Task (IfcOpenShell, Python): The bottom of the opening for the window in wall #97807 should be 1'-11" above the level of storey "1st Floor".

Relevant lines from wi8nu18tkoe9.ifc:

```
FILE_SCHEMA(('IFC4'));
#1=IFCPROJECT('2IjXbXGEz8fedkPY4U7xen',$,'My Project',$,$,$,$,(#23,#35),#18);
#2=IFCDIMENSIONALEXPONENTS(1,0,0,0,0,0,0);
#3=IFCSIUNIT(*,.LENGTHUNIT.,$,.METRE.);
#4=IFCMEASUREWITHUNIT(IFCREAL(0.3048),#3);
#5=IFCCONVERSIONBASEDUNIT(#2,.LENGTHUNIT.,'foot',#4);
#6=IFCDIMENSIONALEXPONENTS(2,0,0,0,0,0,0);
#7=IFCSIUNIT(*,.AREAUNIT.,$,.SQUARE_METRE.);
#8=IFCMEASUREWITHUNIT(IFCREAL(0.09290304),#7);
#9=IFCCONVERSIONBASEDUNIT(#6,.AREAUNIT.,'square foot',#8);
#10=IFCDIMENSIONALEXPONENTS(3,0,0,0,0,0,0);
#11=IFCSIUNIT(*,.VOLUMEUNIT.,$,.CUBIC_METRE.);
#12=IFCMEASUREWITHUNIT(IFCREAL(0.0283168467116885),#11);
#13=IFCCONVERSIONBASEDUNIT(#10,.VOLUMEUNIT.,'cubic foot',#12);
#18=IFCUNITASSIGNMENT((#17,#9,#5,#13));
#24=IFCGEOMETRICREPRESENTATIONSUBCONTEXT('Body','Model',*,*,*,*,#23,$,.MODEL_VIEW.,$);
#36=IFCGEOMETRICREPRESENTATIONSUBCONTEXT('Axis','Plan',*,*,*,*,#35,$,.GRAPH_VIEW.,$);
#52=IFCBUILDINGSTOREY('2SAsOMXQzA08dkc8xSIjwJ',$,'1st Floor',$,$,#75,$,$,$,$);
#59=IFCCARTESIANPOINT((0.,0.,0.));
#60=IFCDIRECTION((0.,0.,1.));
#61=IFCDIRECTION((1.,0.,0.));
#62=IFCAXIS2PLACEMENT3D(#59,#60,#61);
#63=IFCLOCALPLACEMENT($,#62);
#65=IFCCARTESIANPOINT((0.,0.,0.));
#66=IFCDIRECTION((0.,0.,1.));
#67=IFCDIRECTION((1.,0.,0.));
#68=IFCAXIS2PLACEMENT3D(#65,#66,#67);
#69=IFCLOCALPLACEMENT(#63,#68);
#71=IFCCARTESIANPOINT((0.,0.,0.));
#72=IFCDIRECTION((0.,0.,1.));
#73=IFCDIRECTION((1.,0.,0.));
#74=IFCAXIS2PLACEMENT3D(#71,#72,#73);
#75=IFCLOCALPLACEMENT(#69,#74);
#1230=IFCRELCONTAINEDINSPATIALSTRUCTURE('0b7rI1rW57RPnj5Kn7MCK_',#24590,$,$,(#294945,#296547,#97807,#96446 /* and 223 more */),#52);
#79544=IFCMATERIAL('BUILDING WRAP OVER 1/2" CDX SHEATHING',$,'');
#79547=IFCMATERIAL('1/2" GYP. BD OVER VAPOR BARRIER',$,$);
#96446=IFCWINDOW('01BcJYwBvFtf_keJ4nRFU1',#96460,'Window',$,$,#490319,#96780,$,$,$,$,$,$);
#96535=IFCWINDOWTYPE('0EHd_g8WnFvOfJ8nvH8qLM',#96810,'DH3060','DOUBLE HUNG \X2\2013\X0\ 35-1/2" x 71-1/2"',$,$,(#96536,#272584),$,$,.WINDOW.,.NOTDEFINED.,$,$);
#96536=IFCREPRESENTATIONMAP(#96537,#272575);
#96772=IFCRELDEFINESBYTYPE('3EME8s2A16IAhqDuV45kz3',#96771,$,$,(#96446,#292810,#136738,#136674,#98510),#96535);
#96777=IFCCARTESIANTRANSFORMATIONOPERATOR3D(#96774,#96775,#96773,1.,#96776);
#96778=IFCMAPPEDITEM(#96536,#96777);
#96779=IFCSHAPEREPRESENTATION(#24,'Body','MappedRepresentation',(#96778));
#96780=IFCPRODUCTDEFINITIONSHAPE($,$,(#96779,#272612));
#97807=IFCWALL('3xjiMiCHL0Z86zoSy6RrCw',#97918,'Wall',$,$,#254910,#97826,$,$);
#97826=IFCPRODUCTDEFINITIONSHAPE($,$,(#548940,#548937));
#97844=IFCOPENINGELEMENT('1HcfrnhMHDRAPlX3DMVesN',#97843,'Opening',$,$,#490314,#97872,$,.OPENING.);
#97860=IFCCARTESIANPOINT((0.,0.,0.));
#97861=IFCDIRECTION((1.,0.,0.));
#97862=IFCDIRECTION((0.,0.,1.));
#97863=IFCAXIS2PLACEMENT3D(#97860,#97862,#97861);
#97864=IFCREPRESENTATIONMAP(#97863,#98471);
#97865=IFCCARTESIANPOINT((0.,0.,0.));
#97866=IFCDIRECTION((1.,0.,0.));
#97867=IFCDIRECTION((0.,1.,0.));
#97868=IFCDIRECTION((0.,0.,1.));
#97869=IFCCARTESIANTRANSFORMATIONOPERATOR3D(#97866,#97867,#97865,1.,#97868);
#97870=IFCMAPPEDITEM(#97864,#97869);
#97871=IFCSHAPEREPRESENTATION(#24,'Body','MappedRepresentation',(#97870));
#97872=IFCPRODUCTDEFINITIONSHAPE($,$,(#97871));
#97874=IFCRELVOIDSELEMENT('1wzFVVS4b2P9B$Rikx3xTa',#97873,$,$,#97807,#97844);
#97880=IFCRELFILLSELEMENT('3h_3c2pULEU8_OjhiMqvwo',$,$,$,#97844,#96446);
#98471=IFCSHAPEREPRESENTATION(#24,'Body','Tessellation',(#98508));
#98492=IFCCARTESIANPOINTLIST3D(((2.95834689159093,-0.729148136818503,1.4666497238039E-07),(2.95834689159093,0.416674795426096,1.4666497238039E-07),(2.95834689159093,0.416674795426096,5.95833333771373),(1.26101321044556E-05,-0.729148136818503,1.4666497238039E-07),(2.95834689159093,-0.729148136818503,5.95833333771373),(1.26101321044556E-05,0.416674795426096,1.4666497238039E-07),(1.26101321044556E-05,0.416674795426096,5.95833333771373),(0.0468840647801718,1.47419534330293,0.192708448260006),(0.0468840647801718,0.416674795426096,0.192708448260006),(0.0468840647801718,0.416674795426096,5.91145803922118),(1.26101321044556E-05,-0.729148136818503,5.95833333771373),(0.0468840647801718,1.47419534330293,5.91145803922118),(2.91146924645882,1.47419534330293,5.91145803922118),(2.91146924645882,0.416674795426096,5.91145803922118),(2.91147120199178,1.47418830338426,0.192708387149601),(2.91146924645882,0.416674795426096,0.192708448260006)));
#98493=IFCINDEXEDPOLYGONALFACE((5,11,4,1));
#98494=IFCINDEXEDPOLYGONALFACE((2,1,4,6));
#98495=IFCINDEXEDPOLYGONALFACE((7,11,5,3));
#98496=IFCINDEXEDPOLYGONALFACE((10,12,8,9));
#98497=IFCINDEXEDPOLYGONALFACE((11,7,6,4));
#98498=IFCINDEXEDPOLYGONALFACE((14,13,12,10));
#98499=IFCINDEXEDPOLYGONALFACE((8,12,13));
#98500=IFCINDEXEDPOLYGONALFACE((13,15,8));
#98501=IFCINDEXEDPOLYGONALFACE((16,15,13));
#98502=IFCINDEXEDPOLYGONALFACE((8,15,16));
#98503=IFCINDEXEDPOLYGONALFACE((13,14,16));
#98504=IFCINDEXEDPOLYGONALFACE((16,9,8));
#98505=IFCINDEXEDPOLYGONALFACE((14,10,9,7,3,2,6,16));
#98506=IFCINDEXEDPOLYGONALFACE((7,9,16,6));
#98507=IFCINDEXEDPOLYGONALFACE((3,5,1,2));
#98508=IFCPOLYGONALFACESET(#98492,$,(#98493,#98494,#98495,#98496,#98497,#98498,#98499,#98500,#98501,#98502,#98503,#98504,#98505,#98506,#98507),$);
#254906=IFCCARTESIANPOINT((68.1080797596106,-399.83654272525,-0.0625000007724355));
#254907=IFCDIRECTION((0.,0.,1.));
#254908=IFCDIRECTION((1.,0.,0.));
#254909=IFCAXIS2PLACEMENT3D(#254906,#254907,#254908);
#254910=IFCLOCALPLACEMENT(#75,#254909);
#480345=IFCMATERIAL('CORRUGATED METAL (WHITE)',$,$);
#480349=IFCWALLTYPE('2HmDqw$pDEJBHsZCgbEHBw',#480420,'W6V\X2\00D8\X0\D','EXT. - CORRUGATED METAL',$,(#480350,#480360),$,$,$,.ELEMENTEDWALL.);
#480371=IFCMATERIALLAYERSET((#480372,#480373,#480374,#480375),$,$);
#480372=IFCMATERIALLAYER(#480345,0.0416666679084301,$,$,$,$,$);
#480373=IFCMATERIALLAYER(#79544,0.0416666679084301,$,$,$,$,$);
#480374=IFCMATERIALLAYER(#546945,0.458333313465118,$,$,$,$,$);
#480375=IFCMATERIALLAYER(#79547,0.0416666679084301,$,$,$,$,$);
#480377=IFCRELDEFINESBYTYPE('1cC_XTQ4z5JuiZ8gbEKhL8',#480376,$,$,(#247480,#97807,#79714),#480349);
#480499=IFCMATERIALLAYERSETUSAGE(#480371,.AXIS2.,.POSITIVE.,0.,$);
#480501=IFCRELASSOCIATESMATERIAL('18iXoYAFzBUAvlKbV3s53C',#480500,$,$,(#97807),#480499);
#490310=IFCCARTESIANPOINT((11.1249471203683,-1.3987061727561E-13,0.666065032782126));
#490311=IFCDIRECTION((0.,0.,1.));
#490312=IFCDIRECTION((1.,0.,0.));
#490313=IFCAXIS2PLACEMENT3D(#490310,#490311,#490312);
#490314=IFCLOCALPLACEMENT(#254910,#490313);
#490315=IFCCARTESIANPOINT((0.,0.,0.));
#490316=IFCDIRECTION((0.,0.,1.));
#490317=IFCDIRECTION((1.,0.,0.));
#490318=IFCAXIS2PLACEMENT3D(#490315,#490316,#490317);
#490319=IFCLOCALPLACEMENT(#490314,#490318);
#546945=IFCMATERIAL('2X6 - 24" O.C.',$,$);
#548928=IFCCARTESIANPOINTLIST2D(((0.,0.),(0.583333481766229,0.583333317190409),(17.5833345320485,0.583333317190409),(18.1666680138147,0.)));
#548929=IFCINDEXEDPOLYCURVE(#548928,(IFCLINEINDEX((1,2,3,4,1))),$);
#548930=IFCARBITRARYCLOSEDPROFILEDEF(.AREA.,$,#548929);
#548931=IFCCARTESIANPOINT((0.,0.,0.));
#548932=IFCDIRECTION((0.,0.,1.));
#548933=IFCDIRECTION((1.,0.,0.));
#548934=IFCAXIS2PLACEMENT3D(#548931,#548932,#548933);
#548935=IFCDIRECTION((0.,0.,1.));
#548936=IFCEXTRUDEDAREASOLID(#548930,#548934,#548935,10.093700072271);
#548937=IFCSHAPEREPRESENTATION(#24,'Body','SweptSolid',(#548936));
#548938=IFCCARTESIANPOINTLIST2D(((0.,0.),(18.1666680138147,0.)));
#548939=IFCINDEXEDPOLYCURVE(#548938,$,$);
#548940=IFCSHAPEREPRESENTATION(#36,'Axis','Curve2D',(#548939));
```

```python
import numpy as np
import ifcopenshell
import ifcopenshell.api.geometry
import ifcopenshell.geom
import ifcopenshell.util.element
import ifcopenshell.util.placement
import ifcopenshell.util.shape
import ifcopenshell.util.unit

model = ifcopenshell.open("wi8nu18tkoe9.ifc")
unit_scale = ifcopenshell.util.unit.calculate_unit_scale(model)

window = model.by_guid("01BcJYwBvFtf_keJ4nRFU1")
opening = window.FillsVoids[0].RelatingOpeningElement
storey = ifcopenshell.util.element.get_container(window, ifc_class="IfcBuildingStorey")
level = ifcopenshell.util.placement.get_local_placement(storey.ObjectPlacement)[2, 3]

# The opening's origin need not be at the sill, so measure its lowest point.
shape = ifcopenshell.geom.create_shape(ifcopenshell.geom.settings(), opening)
bottom = ifcopenshell.util.shape.get_shape_bottom_elevation(shape, shape.geometry) / unit_scale
dz = level + 23 * 0.0254 / unit_scale - bottom

shift = np.array([0.0, 0.0, dz])
# The window is placed relative to its opening, so it follows when the opening moves.
matrix = ifcopenshell.util.placement.get_local_placement(opening.ObjectPlacement)
matrix[:3, 3] += shift
ifcopenshell.api.geometry.edit_object_placement(
    model, product=opening, matrix=matrix, is_si=False, should_transform_children=True
)

print(f"moved by {dz * unit_scale:+.3f} m")

model.write("wi8nu18tkoe9-out.ifc")
```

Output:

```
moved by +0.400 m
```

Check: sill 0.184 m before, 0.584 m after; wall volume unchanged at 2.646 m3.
